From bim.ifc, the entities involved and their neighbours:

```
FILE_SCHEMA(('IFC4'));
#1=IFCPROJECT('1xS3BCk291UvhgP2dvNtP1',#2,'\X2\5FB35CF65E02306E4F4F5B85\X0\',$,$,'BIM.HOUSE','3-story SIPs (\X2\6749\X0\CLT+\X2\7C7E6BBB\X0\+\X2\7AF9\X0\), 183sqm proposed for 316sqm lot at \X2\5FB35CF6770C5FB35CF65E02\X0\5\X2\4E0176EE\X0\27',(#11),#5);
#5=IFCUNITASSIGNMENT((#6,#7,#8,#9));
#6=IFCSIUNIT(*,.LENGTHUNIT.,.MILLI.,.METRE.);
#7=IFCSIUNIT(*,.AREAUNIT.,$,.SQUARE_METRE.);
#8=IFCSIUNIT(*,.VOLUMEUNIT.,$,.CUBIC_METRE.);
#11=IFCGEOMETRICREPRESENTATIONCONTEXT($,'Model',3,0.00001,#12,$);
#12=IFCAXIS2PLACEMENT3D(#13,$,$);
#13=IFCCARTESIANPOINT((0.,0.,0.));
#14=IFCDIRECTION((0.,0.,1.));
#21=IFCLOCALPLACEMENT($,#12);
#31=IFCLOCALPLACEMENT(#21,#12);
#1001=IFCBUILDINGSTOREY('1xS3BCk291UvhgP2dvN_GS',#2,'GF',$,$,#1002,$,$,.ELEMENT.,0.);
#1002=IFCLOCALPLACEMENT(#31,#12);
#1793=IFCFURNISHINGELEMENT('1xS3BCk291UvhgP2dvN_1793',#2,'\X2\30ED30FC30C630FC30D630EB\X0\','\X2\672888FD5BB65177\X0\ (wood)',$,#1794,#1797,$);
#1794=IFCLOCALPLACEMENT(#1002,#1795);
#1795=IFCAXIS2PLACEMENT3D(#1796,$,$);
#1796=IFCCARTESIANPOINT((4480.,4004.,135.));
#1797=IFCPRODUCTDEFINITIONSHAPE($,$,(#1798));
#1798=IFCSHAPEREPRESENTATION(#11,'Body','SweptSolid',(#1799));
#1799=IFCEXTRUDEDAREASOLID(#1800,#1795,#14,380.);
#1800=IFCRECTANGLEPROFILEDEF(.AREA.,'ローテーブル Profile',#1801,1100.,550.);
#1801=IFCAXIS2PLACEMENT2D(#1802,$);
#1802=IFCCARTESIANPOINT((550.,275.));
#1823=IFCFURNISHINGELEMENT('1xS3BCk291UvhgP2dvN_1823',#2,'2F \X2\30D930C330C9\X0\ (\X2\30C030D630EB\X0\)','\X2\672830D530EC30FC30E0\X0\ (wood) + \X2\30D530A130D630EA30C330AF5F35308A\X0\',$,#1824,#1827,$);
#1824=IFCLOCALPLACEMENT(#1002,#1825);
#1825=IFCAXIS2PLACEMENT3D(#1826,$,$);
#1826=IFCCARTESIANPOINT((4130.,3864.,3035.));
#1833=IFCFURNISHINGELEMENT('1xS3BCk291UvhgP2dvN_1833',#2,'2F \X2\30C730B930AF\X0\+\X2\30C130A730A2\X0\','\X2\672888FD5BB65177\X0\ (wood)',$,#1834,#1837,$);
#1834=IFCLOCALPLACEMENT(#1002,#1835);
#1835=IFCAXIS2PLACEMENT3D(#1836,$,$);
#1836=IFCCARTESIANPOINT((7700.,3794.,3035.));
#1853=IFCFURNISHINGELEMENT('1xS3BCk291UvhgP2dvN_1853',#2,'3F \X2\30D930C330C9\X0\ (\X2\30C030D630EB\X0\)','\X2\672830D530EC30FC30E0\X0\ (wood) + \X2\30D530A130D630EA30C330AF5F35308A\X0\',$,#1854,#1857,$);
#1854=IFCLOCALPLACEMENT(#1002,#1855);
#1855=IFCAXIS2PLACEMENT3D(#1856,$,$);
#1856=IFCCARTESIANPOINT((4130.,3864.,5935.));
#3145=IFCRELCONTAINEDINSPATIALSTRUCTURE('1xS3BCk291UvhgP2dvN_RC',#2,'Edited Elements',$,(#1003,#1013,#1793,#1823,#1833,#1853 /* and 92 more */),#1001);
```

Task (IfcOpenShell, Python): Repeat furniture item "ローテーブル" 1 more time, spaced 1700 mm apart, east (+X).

```python
import numpy as np
import ifcopenshell
import ifcopenshell.api.geometry
import ifcopenshell.api.root
import ifcopenshell.util.element
import ifcopenshell.util.placement

model = ifcopenshell.open("bim.ifc")


def reuse_history(source, copy):
    """copy_class also copies each property set's owner history, people and application; keep the originals."""
    for rel in copy.IsDefinedBy:
        if rel.is_a("IfcRelDefinesByProperties") and (history := rel.RelatingPropertyDefinition.OwnerHistory):
            rel.RelatingPropertyDefinition.OwnerHistory = source.OwnerHistory
            ifcopenshell.util.element.remove_deep2(model, history)


source = model.by_id(1793)
base = ifcopenshell.util.placement.get_local_placement(source.ObjectPlacement)
step = np.array([1.0, 0.0, 0.0]) * 1700.0

for i in range(1, 2):
    copy = ifcopenshell.api.root.copy_class(model, product=source)
    copy.Representation = ifcopenshell.util.element.copy_deep(
        model, source.Representation, exclude=["IfcGeometricRepresentationContext", "IfcRepresentationMap"]
    )
    reuse_history(source, copy)
    matrix = base.copy()
    matrix[:3, 3] += i * step
    print("added at", matrix[:3, 3].round(3) + 0.0)
    ifcopenshell.api.geometry.edit_object_placement(model, product=copy, matrix=matrix, is_si=False)

model.write("bim_v2.ifc")
```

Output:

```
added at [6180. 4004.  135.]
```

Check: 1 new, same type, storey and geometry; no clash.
